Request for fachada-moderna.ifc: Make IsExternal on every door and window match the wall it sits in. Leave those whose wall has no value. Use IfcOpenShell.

First a look at what the model holds.

```python
import ifcopenshell
import ifcopenshell.util.element

model = ifcopenshell.open("fachada-moderna.ifc")
print(model.schema)
seen = {}
for e in model.by_type("IfcDoor") + model.by_type("IfcWindow"):
    if not e.FillsVoids:
        continue
    host = e.FillsVoids[0].RelatingOpeningElement.VoidsElements[0].RelatingBuildingElement
    own = ifcopenshell.util.element.get_pset(e, f"Pset_{e.is_a()[3:].removesuffix('StandardCase')}Common", "IsExternal")
    wall = ifcopenshell.util.element.get_pset(host, "Pset_WallCommon", "IsExternal")
    seen[e.is_a(), own, wall] = seen.get((e.is_a(), own, wall), 0) + 1
for (cls, own, wall), count in sorted(seen.items(), key=str):
    print(count, cls, "IsExternal:", own, "| host wall:", wall)
```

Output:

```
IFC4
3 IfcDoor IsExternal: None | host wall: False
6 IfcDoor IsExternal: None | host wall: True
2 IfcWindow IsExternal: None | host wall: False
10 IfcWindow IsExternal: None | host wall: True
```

```python
import ifcopenshell
import ifcopenshell.api.pset
import ifcopenshell.util.element

model = ifcopenshell.open("fachada-moderna.ifc")

count = 0
for ifc_class, pset_name in (("IfcDoor", "Pset_DoorCommon"), ("IfcWindow", "Pset_WindowCommon")):
    for e in model.by_type(ifc_class):
        if not e.FillsVoids:
            continue
        host = e.FillsVoids[0].RelatingOpeningElement.VoidsElements[0].RelatingBuildingElement
        external = ifcopenshell.util.element.get_pset(host, "Pset_WallCommon", "IsExternal")
        if external is None or ifcopenshell.util.element.get_pset(e, pset_name, "IsExternal") == external:
            continue
        pset = ifcopenshell.api.pset.add_pset(model, product=e, name=pset_name)
        ifcopenshell.api.pset.edit_pset(model, pset=pset, properties={"IsExternal": external})
        count += 1

print(count, "updated")

model.write("fachada-moderna_updated.ifc")
```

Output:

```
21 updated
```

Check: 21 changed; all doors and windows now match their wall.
